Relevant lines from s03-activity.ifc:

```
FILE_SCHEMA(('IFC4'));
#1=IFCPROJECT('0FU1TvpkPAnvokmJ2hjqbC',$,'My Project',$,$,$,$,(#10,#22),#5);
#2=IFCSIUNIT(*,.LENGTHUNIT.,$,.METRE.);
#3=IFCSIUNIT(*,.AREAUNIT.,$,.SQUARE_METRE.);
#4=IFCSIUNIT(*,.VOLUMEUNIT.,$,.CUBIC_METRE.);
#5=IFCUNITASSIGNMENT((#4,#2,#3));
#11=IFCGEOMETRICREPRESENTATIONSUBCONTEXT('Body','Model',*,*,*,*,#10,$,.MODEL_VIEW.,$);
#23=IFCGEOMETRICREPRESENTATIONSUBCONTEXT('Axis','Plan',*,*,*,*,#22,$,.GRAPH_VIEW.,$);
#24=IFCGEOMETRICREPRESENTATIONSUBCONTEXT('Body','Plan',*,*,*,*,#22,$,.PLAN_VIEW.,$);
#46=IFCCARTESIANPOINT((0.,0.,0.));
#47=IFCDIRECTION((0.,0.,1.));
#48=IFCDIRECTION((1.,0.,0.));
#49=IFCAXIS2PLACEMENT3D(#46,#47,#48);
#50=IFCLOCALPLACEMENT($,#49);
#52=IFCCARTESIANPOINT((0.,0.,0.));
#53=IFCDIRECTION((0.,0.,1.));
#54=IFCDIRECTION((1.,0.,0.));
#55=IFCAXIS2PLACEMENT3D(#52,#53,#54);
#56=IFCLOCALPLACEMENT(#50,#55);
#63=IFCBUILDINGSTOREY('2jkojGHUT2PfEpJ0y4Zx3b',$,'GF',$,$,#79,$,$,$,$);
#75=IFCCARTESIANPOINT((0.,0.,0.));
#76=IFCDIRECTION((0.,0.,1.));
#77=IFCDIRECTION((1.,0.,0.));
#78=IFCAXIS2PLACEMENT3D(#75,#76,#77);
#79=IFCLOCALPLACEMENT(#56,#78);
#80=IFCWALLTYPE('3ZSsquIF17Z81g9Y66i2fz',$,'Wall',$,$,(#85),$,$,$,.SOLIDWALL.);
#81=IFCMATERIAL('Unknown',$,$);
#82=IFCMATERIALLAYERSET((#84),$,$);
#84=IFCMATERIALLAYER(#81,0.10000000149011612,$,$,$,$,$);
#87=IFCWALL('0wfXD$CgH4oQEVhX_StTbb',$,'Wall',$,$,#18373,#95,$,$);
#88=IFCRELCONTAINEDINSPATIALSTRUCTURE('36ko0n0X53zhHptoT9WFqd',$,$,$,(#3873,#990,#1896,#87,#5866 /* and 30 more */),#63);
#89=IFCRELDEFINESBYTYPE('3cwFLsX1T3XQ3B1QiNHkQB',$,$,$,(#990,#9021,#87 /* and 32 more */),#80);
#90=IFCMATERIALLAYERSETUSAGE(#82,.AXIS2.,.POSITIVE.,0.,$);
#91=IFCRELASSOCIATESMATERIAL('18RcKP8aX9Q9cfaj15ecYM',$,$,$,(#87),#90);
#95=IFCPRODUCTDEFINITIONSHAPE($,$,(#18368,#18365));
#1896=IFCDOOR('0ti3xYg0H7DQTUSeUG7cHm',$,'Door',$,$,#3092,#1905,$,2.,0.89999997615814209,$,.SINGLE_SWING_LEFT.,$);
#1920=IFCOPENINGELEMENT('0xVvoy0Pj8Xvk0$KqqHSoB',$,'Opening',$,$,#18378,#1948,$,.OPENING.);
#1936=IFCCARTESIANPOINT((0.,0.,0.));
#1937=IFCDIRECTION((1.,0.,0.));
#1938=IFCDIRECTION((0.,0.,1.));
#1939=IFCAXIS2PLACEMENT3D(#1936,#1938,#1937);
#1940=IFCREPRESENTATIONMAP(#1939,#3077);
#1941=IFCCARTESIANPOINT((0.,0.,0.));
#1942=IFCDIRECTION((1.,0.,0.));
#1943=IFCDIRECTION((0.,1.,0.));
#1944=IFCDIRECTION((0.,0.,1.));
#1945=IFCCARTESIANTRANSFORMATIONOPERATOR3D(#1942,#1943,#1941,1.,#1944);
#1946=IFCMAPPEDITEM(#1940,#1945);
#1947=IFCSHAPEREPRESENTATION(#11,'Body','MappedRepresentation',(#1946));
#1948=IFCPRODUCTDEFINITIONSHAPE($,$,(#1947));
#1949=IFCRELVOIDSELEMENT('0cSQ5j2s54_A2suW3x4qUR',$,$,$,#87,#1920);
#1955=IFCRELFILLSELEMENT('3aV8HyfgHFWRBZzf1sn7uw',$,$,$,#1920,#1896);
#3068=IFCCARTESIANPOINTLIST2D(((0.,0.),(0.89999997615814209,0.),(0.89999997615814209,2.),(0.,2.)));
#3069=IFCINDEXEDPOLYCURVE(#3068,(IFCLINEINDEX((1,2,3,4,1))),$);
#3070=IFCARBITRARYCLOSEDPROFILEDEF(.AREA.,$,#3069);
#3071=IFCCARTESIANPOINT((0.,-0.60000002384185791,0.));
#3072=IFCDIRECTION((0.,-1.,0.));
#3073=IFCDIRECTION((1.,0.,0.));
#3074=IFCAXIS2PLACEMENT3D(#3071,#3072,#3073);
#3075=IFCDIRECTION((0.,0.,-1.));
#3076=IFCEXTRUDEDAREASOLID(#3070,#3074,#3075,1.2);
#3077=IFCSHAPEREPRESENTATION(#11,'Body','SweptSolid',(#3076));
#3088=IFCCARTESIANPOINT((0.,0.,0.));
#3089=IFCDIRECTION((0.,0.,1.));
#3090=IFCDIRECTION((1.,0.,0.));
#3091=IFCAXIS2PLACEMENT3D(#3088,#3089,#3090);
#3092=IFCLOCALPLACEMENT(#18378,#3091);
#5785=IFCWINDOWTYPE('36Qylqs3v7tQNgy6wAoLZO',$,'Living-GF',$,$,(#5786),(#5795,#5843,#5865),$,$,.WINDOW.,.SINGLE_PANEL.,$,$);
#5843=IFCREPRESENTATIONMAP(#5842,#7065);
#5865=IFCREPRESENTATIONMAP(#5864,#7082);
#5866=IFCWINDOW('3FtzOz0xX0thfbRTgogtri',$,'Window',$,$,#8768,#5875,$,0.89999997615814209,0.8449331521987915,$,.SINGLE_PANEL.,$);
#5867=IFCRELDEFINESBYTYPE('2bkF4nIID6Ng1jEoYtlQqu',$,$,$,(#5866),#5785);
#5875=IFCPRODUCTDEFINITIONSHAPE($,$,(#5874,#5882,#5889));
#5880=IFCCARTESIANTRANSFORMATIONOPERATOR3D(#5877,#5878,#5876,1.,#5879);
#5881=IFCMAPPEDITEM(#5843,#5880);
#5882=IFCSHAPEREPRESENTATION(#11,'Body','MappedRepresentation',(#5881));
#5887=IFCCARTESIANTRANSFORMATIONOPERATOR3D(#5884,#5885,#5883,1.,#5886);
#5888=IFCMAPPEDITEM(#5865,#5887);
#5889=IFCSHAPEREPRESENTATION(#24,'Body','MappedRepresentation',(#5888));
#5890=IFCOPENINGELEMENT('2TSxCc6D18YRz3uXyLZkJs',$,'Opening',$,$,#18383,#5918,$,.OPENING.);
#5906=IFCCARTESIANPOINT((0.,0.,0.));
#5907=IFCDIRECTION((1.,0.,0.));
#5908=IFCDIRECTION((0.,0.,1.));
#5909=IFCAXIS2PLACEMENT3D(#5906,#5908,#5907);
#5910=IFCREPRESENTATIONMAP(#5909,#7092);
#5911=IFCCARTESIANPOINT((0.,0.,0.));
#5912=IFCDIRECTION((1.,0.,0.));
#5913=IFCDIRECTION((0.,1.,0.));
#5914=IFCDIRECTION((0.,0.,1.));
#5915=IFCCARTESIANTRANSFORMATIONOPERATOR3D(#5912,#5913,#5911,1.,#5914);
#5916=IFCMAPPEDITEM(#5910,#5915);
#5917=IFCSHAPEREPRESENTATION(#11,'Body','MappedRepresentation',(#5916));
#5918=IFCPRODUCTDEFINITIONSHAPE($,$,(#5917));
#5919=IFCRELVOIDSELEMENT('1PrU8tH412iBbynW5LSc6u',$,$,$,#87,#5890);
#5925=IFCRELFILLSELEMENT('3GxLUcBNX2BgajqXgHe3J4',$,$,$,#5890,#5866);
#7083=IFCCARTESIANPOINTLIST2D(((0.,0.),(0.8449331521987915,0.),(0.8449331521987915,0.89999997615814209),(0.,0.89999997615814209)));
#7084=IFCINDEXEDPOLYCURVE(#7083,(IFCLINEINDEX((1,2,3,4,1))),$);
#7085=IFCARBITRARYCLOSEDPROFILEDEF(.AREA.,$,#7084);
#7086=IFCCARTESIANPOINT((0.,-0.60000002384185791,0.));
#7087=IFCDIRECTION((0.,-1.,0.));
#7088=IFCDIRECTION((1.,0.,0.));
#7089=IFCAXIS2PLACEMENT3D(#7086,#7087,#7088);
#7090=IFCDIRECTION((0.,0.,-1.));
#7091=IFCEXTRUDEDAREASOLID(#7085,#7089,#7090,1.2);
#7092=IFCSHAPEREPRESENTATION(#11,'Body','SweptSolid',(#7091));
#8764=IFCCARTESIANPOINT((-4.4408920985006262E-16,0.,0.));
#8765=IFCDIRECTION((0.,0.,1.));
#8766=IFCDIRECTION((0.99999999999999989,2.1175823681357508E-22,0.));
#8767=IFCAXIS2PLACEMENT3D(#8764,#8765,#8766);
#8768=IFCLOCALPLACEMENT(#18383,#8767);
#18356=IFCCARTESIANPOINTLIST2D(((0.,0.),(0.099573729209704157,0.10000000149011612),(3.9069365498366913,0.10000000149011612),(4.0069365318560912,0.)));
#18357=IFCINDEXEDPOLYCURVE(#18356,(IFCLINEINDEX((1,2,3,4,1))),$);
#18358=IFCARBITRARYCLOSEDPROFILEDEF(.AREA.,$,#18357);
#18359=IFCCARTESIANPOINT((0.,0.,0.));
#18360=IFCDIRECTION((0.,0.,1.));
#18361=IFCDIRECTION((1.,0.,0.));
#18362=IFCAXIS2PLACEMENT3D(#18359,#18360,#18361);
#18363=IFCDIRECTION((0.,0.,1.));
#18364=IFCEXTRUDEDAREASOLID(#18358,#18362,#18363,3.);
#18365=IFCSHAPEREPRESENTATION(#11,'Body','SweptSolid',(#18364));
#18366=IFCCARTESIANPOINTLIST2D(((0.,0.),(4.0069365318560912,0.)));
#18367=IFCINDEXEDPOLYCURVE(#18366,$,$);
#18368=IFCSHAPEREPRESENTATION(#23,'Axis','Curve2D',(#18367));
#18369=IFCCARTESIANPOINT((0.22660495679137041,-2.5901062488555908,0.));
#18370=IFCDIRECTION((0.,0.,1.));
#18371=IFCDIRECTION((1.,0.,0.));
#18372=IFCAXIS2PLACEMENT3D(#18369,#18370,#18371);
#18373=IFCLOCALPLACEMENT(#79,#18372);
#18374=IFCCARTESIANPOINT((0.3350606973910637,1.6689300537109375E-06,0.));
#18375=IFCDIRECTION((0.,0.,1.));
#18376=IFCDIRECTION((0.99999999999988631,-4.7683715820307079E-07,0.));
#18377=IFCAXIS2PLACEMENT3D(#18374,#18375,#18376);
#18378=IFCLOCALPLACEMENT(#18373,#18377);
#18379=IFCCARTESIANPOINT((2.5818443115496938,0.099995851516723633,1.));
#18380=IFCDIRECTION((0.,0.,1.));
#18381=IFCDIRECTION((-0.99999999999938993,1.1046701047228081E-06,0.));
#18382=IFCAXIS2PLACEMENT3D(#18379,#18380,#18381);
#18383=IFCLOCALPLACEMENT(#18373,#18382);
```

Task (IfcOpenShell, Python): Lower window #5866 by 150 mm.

```python
import numpy as np
import ifcopenshell
import ifcopenshell.api.geometry
import ifcopenshell.util.placement
import ifcopenshell.util.unit

model = ifcopenshell.open("s03-activity.ifc")
unit_scale = ifcopenshell.util.unit.calculate_unit_scale(model)

window = model.by_guid("3FtzOz0xX0thfbRTgogtri")
opening = window.FillsVoids[0].RelatingOpeningElement
dz = -0.15

shift = np.array([0.0, 0.0, dz])
# The window is placed relative to its opening, so it follows when the opening moves.
matrix = ifcopenshell.util.placement.get_local_placement(opening.ObjectPlacement)
matrix[:3, 3] += shift
ifcopenshell.api.geometry.edit_object_placement(
    model, product=opening, matrix=matrix, is_si=False, should_transform_children=True
)

print(f"moved by {dz * unit_scale:+.3f} m")

model.write("s03-activity_edited.ifc")
```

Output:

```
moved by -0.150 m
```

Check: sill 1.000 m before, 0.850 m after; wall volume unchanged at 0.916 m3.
